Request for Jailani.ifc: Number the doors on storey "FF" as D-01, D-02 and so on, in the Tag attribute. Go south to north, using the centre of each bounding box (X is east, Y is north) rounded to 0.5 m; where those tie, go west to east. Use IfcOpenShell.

First a look at what the model holds.

```python
import ifcopenshell
import ifcopenshell.util.element
import ifcopenshell.util.placement

model = ifcopenshell.open("Jailani.ifc")
print(model.schema)
storey = next(s for s in model.by_type("IfcBuildingStorey") if s.Name == "FF")
doors = [e for e in ifcopenshell.util.element.get_decomposition(storey) if e.is_a("IfcDoor")]
for e in sorted(doors, key=lambda e: e.id()):
    origin = ifcopenshell.util.placement.get_local_placement(e.ObjectPlacement)[:3, 3]
    print(e.id(), e.Tag, e.Name, origin.round(2) + 0.0, sep=" | ")
```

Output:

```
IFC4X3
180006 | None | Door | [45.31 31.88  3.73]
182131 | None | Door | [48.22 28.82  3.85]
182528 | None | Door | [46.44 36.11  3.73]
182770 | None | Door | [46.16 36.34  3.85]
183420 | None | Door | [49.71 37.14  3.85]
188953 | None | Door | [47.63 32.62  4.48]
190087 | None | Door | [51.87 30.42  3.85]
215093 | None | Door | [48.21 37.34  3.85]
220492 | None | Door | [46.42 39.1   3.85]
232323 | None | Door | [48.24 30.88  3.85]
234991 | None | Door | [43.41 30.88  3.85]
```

```python
import ifcopenshell
import ifcopenshell.geom
import ifcopenshell.util.element
import ifcopenshell.util.shape

model = ifcopenshell.open("Jailani.ifc")
settings = ifcopenshell.geom.settings()
settings.set("use-world-coords", True)


def centre(element):
    shape = ifcopenshell.geom.create_shape(settings, element)
    return ifcopenshell.util.shape.get_bbox_centroid(shape.geometry)


storey = next(s for s in model.by_type("IfcBuildingStorey") if s.Name == "FF")
doors = [e for e in ifcopenshell.util.element.get_decomposition(storey) if e.is_a("IfcDoor")]

# Insertion points can sit at a corner or the storey origin, so sort by the geometry (in metres).
centres = {e: centre(e) for e in doors}
doors.sort(key=lambda e: (round(centres[e][1] / 0.5), centres[e][0]))

for i, e in enumerate(doors, start=1):
    number = f"D-{i:02d}"
    e.Tag = number
    print(e.id(), number)

model.write("Jailani_rev.ifc")
```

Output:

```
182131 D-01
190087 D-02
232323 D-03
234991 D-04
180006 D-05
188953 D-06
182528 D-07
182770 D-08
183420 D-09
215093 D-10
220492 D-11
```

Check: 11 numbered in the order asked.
